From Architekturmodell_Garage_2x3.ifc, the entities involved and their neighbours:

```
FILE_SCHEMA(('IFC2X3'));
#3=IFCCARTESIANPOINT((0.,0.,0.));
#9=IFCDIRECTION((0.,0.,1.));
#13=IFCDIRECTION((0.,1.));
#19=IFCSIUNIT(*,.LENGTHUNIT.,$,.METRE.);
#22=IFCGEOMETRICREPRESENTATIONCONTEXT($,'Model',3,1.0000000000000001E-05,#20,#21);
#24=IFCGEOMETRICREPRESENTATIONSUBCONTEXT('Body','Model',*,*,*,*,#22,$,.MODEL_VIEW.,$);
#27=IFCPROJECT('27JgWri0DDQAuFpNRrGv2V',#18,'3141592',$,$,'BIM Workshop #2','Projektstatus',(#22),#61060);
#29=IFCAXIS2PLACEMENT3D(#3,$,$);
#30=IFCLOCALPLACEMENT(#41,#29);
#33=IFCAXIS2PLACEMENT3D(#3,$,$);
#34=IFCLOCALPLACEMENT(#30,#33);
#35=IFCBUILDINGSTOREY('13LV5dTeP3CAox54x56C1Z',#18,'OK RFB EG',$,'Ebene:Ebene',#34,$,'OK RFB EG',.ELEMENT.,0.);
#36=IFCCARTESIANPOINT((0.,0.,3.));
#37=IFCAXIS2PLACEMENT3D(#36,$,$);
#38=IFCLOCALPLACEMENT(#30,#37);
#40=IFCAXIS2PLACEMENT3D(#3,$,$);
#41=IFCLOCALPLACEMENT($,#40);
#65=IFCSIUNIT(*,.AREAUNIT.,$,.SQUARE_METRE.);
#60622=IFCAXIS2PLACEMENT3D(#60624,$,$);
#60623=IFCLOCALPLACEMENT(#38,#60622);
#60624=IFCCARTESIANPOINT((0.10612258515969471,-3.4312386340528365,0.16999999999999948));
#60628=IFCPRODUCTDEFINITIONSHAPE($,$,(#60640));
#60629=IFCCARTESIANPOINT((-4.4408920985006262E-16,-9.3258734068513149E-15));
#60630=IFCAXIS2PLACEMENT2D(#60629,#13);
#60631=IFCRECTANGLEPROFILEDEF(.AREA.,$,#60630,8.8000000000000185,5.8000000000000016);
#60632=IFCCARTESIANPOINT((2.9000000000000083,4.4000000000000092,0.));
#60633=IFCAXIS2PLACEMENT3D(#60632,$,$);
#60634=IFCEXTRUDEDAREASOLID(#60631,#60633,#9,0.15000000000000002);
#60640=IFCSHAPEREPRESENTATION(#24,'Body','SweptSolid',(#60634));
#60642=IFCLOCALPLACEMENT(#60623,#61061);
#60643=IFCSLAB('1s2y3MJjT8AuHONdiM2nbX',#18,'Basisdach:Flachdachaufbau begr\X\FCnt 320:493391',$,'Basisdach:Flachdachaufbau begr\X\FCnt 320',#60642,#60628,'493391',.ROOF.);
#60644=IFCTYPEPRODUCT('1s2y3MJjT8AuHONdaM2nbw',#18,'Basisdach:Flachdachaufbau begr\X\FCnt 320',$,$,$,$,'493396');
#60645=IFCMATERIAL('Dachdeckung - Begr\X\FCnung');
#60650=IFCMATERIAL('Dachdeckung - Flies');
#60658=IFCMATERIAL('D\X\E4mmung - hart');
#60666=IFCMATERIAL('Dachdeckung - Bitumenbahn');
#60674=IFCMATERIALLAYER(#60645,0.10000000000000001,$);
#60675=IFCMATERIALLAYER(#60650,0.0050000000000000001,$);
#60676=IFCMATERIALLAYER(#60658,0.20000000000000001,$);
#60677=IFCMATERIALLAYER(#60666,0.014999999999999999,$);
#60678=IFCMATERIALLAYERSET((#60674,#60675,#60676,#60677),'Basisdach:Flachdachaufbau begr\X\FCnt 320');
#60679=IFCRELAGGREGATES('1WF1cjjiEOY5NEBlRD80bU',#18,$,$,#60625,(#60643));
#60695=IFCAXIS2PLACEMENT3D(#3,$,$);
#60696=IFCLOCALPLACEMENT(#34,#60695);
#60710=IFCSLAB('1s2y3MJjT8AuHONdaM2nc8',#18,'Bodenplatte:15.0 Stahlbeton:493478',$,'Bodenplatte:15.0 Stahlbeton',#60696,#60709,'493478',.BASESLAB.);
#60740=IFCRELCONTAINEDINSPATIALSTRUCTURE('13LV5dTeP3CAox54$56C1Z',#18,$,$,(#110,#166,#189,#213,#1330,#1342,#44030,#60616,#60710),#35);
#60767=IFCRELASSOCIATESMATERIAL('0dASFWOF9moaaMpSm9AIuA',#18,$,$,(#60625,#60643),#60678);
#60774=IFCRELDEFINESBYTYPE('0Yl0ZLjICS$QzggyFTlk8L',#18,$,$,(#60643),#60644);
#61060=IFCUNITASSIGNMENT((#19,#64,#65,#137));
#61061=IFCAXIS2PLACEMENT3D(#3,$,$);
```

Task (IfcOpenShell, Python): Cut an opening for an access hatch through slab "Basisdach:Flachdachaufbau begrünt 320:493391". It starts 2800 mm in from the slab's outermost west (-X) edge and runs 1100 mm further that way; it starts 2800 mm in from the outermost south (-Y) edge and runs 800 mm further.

```python
import numpy as np
import ifcopenshell
import ifcopenshell.api.feature
import ifcopenshell.api.geometry
import ifcopenshell.api.root
import ifcopenshell.geom
import ifcopenshell.util.placement
import ifcopenshell.util.representation
import ifcopenshell.util.shape
import ifcopenshell.util.unit

model = ifcopenshell.open("Architekturmodell_Garage_2x3.ifc")
unit_scale = ifcopenshell.util.unit.calculate_unit_scale(model)
settings = ifcopenshell.geom.settings()


def volume(element):
    """Net volume in cubic metres, openings subtracted."""
    shape = ifcopenshell.geom.create_shape(settings, element)
    return ifcopenshell.util.shape.get_volume(shape.geometry)


slab = model.by_guid("1s2y3MJjT8AuHONdiM2nbX")
before = volume(slab)

# Extent in the slab's own axes, in metres. The edges named are its -X and -Y sides.
slab_shape = ifcopenshell.geom.create_shape(settings, slab)
vertices = ifcopenshell.util.shape.get_vertices(slab_shape.geometry)
x_min, y_min, bottom = vertices.min(axis=0)
top = vertices[:, 2].max()

opening = ifcopenshell.api.root.create_entity(model, ifc_class="IfcOpeningElement", name="Access hatch opening")
context = ifcopenshell.util.representation.get_context(model, "Model", "Body", "MODEL_VIEW")
width, depth = 1.1, 0.8
outline = [(0.0, 0.0), (width, 0.0), (width, depth), (0.0, depth), (0.0, 0.0)]
# Overshoot both faces by 50 mm so the cut is clean.
shape = ifcopenshell.api.geometry.add_slab_representation(
    model, context=context, depth=top - bottom + 0.1, polyline=outline
)
ifcopenshell.api.geometry.assign_representation(model, product=opening, representation=shape)

matrix = ifcopenshell.util.placement.get_local_placement(slab.ObjectPlacement)
matrix[:, 3] = matrix @ np.append(np.array([x_min + 2.8, y_min + 2.8, bottom - 0.05]) / unit_scale, 1.0)
ifcopenshell.api.geometry.edit_object_placement(model, product=opening, matrix=matrix, is_si=False)
ifcopenshell.api.feature.add_feature(model, feature=opening, element=slab)

after = volume(slab)

print(f"slab volume {before:.3f} -> {after:.3f} m3")

model.write("Architekturmodell_Garage_2x3-out.ifc")
```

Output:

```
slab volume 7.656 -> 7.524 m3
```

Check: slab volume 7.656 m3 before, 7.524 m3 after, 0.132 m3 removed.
